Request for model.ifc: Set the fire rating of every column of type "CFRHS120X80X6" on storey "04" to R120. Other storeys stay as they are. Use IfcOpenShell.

First a look at what the model holds.

```python
import ifcopenshell
import ifcopenshell.util.element

model = ifcopenshell.open("model.ifc")
print(model.schema)
storey = next(s for s in model.by_type("IfcBuildingStorey") if s.Name == "04")
columns = [e for e in ifcopenshell.util.element.get_decomposition(storey) if e.is_a("IfcColumn")]
seen = {}
for e in columns:
    element_type = ifcopenshell.util.element.get_type(e)
    key = (element_type.Name if element_type != e and element_type else None, ifcopenshell.util.element.get_pset(e, "Pset_ColumnCommon", "FireRating"))
    seen[key] = seen.get(key, 0) + 1
for (name, value), count in sorted(seen.items(), key=str):
    print(count, "x", name, "|", value)
```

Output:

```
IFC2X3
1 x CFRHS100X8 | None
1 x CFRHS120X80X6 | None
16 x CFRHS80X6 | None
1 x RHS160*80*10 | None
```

```python
import ifcopenshell
import ifcopenshell.api.pset
import ifcopenshell.util.element

model = ifcopenshell.open("model.ifc")

storey = next(s for s in model.by_type("IfcBuildingStorey") if s.Name == "04")
columns = [e for e in ifcopenshell.util.element.get_decomposition(storey) if e.is_a("IfcColumn")]

count = 0
for e in columns:
    element_type = ifcopenshell.util.element.get_type(e)
    if element_type in (None, e) or element_type.Name != "CFRHS120X80X6":
        continue
    # add_pset returns the element's existing set when there is one.
    pset = ifcopenshell.api.pset.add_pset(model, product=e, name="Pset_ColumnCommon")
    ifcopenshell.api.pset.edit_pset(model, pset=pset, properties={"FireRating": "R120"})
    count += 1

print(count, "columns updated")

model.write("model_v2.ifc")
```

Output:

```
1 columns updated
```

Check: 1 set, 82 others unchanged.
